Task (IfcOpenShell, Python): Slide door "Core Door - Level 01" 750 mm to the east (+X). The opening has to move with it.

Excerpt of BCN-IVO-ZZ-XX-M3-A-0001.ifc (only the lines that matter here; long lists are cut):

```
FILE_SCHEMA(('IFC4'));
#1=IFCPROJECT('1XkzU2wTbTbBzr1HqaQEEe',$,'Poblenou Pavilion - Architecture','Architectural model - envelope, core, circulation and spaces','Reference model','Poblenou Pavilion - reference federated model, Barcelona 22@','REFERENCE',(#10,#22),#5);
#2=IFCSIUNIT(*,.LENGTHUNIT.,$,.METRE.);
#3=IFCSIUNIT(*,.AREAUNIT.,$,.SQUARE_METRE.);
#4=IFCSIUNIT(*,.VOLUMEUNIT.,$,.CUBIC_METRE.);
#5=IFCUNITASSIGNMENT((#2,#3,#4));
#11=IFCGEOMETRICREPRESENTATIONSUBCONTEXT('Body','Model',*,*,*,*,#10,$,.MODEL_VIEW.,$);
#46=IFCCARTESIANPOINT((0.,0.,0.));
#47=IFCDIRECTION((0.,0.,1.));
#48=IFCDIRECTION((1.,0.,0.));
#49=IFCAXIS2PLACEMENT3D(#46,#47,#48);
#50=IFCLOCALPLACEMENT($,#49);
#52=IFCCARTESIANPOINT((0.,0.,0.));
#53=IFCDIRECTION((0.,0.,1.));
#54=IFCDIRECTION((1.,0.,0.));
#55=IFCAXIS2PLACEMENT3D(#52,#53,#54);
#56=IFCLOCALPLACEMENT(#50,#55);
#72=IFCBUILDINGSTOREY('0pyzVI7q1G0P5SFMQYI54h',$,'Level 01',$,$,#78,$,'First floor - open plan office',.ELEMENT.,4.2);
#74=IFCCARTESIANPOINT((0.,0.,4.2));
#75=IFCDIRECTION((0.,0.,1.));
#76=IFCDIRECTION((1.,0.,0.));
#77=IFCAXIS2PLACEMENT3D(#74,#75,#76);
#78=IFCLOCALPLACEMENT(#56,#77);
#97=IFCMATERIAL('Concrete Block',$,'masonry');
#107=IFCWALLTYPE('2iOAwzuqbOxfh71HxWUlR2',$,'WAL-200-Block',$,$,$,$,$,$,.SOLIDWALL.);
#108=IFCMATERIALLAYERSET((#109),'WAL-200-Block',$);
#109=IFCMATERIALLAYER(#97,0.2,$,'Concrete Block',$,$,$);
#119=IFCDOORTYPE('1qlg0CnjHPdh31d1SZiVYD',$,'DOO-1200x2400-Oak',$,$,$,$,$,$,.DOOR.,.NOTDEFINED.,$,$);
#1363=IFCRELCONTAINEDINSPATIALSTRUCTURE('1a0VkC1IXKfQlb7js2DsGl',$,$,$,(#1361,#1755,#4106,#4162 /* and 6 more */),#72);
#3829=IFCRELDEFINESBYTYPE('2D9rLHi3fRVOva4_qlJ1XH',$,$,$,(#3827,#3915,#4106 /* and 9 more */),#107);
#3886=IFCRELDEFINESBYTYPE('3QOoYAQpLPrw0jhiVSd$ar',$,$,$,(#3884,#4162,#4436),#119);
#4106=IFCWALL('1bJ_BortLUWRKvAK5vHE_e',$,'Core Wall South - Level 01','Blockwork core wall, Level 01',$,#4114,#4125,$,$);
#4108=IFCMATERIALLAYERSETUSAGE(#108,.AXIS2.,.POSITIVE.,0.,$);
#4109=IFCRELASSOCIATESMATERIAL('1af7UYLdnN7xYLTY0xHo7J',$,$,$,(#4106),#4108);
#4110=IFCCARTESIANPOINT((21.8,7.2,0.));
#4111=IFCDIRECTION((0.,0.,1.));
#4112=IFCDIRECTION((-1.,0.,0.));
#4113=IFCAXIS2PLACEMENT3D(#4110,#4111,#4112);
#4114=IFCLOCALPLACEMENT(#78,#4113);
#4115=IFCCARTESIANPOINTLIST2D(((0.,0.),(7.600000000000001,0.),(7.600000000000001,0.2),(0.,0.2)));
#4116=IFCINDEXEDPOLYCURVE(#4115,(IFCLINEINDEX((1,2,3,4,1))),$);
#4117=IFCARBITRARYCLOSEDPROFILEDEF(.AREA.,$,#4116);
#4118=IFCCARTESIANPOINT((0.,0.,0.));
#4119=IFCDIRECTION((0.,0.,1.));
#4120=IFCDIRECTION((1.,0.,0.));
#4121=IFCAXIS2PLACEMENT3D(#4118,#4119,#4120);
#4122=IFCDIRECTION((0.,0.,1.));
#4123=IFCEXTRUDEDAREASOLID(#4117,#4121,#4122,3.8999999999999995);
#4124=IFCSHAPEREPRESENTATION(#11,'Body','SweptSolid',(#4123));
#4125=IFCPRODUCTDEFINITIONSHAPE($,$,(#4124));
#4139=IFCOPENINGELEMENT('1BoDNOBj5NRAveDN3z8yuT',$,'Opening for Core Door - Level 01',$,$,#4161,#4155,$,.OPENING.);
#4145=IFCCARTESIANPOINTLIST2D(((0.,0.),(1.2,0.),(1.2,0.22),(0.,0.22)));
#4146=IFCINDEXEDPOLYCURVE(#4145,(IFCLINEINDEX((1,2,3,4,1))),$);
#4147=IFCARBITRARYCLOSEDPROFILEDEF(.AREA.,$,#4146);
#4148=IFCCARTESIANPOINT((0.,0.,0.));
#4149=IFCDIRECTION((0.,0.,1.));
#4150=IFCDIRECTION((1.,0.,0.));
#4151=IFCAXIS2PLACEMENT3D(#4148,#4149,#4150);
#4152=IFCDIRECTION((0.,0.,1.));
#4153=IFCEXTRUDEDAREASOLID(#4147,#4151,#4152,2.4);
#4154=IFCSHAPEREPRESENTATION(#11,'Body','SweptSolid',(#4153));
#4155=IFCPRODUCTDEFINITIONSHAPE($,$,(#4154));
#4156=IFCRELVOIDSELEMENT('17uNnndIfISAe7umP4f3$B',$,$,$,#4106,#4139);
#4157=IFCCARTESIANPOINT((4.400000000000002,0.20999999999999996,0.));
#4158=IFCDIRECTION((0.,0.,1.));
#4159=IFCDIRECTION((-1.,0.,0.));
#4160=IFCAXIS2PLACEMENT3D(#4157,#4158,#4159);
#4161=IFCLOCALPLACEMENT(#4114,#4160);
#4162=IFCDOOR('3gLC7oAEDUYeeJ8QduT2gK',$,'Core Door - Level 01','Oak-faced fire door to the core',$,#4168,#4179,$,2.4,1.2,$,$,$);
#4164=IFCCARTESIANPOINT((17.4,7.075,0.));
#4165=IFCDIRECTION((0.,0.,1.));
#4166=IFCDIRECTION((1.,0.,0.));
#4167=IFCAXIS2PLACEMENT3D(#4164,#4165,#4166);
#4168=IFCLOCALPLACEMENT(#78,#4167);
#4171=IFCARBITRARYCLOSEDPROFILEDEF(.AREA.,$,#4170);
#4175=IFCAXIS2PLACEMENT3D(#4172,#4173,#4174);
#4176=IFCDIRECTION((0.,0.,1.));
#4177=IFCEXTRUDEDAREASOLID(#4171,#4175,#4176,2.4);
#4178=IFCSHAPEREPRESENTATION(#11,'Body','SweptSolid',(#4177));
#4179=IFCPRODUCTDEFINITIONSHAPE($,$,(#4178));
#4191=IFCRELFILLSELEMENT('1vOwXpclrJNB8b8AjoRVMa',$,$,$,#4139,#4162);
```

```python
import ifcopenshell
import ifcopenshell.api.geometry
import ifcopenshell.util.placement
import ifcopenshell.util.unit

model = ifcopenshell.open("BCN-IVO-ZZ-XX-M3-A-0001.ifc")
unit_scale = ifcopenshell.util.unit.calculate_unit_scale(model)

door = model.by_id(4162)
opening = door.FillsVoids[0].RelatingOpeningElement
wall = opening.VoidsElements[0].RelatingBuildingElement

wall_matrix = ifcopenshell.util.placement.get_local_placement(wall.ObjectPlacement)
shift = wall_matrix[:3, 0] * -0.75 / unit_scale
before = ifcopenshell.util.placement.get_local_placement(door.ObjectPlacement)[:3, 3].copy()

# The door is not placed relative to its opening, so move both.
for product in (opening, door):
    matrix = ifcopenshell.util.placement.get_local_placement(product.ObjectPlacement)
    matrix[:3, 3] += shift
    ifcopenshell.api.geometry.edit_object_placement(model, product=product, matrix=matrix, is_si=False)

after = ifcopenshell.util.placement.get_local_placement(door.ObjectPlacement)[:3, 3]
print("door moved by", (after - before).round(3) + 0.0)

model.write("BCN-IVO-ZZ-XX-M3-A-0001_rev.ifc")
```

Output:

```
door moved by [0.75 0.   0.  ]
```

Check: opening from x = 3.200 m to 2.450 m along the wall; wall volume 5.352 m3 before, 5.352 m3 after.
